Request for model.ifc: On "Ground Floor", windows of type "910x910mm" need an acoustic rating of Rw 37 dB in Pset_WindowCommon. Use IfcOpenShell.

First a look at what the model holds.

```python
import ifcopenshell
import ifcopenshell.util.element

model = ifcopenshell.open("model.ifc")
print(model.schema)
storey = next(s for s in model.by_type("IfcBuildingStorey") if s.Name == "Ground Floor")
windows = [e for e in ifcopenshell.util.element.get_decomposition(storey) if e.is_a("IfcWindow")]
seen = {}
for e in windows:
    element_type = ifcopenshell.util.element.get_type(e)
    key = (element_type.Name if element_type != e and element_type else None, ifcopenshell.util.element.get_pset(e, "Pset_WindowCommon", "AcousticRating"))
    seen[key] = seen.get(key, 0) + 1
for (name, value), count in sorted(seen.items(), key=str):
    print(count, "x", name, "|", value)
```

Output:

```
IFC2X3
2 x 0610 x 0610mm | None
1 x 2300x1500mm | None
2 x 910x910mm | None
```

```python
import ifcopenshell
import ifcopenshell.api.pset
import ifcopenshell.util.element

model = ifcopenshell.open("model.ifc")

storey = next(s for s in model.by_type("IfcBuildingStorey") if s.Name == "Ground Floor")
windows = [e for e in ifcopenshell.util.element.get_decomposition(storey) if e.is_a("IfcWindow")]

count = 0
for e in windows:
    element_type = ifcopenshell.util.element.get_type(e)
    if element_type in (None, e) or element_type.Name != "910x910mm":
        continue
    # add_pset returns the element's existing set when there is one.
    pset = ifcopenshell.api.pset.add_pset(model, product=e, name="Pset_WindowCommon")
    ifcopenshell.api.pset.edit_pset(model, pset=pset, properties={"AcousticRating": "Rw 37 dB"})
    count += 1

print(count, "windows updated")

model.write("model_v2.ifc")
```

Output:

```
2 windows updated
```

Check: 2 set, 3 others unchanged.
